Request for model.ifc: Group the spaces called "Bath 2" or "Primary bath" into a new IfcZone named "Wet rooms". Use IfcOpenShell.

First a look at what the model holds.

```python
import ifcopenshell

model = ifcopenshell.open("model.ifc")
print(model.schema)
seen = {}
for space in model.by_type("IfcSpace"):
    seen[space.LongName] = seen.get(space.LongName, 0) + 1
for name, count in sorted(seen.items(), key=str):
    print(count, "x", name)
print("zones:", [z.Name for z in model.by_type("IfcZone")][:20])
```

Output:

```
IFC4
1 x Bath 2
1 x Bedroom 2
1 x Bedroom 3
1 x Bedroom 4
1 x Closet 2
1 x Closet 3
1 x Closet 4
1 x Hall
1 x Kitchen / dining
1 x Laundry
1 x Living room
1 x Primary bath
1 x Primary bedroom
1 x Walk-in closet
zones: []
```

```python
import ifcopenshell
import ifcopenshell.api.group
import ifcopenshell.api.root

model = ifcopenshell.open("model.ifc")

names = {"Bath 2", "Primary bath"}
spaces = [s for s in model.by_type("IfcSpace") if s.LongName in names]

zone = ifcopenshell.api.root.create_entity(model, ifc_class="IfcZone", name="Wet rooms")
ifcopenshell.api.group.assign_group(model, products=spaces, group=zone)
print(len(spaces), "spaces in", zone.Name)

model.write("model_updated.ifc")
```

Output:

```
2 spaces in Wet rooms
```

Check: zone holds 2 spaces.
